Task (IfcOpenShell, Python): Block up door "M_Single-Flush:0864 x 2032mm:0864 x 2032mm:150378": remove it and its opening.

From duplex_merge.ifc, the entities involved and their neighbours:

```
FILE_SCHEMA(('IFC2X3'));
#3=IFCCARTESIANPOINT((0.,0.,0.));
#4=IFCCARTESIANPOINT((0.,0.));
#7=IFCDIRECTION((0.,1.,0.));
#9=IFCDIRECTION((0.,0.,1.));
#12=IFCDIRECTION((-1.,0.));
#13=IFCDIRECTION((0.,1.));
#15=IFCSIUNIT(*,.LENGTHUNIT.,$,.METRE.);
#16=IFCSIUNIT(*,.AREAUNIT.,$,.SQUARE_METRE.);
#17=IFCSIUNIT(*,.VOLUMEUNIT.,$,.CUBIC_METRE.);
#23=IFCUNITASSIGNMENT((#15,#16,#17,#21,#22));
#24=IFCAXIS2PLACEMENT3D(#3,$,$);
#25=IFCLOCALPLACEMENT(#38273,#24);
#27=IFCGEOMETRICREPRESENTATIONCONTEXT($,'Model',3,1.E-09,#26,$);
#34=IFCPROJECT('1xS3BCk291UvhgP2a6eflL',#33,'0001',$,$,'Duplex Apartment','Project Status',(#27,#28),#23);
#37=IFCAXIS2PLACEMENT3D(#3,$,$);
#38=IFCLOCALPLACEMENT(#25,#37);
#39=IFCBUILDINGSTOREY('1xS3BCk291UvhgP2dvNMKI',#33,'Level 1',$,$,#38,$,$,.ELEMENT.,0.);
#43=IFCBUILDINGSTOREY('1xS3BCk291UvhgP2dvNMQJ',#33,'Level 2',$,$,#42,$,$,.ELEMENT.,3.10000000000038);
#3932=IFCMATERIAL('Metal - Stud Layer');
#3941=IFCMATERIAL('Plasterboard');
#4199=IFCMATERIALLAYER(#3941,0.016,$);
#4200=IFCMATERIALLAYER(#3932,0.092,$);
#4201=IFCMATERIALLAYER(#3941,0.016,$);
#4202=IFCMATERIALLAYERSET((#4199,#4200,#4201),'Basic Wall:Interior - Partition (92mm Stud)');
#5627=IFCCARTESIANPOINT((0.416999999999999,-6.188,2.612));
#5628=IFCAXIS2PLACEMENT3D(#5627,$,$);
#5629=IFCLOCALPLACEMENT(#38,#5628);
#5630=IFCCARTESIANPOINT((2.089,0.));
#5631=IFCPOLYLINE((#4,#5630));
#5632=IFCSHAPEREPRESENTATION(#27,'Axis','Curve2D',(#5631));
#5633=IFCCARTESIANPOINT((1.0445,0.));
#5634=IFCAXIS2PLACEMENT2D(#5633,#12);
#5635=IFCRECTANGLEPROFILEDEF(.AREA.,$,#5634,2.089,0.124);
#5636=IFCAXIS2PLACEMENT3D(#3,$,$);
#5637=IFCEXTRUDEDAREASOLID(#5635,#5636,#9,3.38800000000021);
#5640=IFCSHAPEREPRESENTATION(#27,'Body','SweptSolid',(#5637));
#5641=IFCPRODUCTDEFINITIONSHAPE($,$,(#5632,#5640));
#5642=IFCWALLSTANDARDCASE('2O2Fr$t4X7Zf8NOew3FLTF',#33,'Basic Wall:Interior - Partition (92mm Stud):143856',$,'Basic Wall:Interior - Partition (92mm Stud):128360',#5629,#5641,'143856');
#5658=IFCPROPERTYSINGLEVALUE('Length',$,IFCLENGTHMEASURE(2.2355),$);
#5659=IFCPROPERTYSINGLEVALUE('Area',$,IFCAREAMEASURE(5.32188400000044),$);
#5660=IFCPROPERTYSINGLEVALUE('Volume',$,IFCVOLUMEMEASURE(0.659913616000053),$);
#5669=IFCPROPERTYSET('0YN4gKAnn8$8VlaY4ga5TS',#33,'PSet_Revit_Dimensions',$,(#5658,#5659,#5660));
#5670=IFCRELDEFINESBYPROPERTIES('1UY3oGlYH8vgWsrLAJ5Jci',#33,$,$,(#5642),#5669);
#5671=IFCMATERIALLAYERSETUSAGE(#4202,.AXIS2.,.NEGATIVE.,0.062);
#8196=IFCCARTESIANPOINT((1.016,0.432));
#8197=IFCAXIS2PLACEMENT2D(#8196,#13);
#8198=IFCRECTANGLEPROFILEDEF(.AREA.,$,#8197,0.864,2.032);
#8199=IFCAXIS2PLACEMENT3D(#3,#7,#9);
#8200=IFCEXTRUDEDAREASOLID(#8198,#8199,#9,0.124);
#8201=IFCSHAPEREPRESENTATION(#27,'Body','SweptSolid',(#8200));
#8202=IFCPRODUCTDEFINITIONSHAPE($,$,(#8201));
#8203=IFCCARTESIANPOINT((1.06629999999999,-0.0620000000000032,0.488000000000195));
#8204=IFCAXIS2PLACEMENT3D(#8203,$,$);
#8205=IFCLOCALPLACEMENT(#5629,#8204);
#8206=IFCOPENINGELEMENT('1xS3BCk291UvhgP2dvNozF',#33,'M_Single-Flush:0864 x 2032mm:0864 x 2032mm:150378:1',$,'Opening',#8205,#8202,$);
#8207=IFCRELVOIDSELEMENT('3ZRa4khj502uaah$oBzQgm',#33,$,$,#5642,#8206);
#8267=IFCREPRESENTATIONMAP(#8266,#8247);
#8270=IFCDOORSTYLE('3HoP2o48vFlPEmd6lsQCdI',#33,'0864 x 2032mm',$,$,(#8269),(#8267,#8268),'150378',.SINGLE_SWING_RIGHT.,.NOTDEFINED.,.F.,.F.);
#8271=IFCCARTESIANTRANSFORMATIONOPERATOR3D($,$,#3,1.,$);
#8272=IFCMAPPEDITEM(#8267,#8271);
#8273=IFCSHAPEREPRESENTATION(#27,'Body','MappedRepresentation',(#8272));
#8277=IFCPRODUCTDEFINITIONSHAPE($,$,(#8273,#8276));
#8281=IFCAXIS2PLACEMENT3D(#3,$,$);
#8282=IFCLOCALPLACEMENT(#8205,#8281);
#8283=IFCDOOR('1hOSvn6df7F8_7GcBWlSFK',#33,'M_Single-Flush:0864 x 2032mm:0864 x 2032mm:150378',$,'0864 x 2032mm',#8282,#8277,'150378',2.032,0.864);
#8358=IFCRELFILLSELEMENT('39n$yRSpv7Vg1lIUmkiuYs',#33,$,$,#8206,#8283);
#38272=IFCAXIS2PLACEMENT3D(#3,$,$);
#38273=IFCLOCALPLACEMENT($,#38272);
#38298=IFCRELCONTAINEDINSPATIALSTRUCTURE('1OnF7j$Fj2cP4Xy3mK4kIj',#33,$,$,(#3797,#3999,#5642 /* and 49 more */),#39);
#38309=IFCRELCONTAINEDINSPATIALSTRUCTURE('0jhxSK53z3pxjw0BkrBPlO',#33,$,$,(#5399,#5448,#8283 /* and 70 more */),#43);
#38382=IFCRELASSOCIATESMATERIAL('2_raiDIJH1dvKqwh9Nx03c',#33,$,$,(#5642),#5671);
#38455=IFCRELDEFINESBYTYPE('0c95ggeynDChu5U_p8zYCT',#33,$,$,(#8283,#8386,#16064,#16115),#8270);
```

```python
import ifcopenshell
import ifcopenshell.api.feature
import ifcopenshell.api.pset
import ifcopenshell.api.root
import ifcopenshell.geom
import ifcopenshell.util.element
import ifcopenshell.util.shape
import ifcopenshell.util.unit

model = ifcopenshell.open("duplex_merge.ifc")
area_scale = ifcopenshell.util.unit.calculate_unit_scale(model, "AREAUNIT")
volume_scale = ifcopenshell.util.unit.calculate_unit_scale(model, "VOLUMEUNIT")
settings = ifcopenshell.geom.settings()


def volume(element):
    """Net volume in cubic metres, openings subtracted."""
    shape = ifcopenshell.geom.create_shape(settings, element)
    return ifcopenshell.util.shape.get_volume(shape.geometry)


door = model.by_id(8283)
opening = door.FillsVoids[0].RelatingOpeningElement
wall = opening.VoidsElements[0].RelatingBuildingElement
before = volume(wall)

ifcopenshell.api.root.remove_product(model, product=door)
ifcopenshell.api.feature.remove_feature(model, feature=opening)

after = volume(wall)
thickness = 0.124  # wall thickness in metres

# Update the wall's stored quantities.
pset = model.by_id(ifcopenshell.util.element.get_pset(wall, "PSet_Revit_Dimensions", should_inherit=False)["id"])
ifcopenshell.api.pset.edit_pset(model, pset=pset, properties={
    "Area": model.create_entity("IfcAreaMeasure", after / thickness / area_scale),
    "Volume": model.create_entity("IfcVolumeMeasure", after / volume_scale),
})

print(f"wall volume {before:.3f} -> {after:.3f} m3")

model.write("duplex_merge_rev.ifc")
```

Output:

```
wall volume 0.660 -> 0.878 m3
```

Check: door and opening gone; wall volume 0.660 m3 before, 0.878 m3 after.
